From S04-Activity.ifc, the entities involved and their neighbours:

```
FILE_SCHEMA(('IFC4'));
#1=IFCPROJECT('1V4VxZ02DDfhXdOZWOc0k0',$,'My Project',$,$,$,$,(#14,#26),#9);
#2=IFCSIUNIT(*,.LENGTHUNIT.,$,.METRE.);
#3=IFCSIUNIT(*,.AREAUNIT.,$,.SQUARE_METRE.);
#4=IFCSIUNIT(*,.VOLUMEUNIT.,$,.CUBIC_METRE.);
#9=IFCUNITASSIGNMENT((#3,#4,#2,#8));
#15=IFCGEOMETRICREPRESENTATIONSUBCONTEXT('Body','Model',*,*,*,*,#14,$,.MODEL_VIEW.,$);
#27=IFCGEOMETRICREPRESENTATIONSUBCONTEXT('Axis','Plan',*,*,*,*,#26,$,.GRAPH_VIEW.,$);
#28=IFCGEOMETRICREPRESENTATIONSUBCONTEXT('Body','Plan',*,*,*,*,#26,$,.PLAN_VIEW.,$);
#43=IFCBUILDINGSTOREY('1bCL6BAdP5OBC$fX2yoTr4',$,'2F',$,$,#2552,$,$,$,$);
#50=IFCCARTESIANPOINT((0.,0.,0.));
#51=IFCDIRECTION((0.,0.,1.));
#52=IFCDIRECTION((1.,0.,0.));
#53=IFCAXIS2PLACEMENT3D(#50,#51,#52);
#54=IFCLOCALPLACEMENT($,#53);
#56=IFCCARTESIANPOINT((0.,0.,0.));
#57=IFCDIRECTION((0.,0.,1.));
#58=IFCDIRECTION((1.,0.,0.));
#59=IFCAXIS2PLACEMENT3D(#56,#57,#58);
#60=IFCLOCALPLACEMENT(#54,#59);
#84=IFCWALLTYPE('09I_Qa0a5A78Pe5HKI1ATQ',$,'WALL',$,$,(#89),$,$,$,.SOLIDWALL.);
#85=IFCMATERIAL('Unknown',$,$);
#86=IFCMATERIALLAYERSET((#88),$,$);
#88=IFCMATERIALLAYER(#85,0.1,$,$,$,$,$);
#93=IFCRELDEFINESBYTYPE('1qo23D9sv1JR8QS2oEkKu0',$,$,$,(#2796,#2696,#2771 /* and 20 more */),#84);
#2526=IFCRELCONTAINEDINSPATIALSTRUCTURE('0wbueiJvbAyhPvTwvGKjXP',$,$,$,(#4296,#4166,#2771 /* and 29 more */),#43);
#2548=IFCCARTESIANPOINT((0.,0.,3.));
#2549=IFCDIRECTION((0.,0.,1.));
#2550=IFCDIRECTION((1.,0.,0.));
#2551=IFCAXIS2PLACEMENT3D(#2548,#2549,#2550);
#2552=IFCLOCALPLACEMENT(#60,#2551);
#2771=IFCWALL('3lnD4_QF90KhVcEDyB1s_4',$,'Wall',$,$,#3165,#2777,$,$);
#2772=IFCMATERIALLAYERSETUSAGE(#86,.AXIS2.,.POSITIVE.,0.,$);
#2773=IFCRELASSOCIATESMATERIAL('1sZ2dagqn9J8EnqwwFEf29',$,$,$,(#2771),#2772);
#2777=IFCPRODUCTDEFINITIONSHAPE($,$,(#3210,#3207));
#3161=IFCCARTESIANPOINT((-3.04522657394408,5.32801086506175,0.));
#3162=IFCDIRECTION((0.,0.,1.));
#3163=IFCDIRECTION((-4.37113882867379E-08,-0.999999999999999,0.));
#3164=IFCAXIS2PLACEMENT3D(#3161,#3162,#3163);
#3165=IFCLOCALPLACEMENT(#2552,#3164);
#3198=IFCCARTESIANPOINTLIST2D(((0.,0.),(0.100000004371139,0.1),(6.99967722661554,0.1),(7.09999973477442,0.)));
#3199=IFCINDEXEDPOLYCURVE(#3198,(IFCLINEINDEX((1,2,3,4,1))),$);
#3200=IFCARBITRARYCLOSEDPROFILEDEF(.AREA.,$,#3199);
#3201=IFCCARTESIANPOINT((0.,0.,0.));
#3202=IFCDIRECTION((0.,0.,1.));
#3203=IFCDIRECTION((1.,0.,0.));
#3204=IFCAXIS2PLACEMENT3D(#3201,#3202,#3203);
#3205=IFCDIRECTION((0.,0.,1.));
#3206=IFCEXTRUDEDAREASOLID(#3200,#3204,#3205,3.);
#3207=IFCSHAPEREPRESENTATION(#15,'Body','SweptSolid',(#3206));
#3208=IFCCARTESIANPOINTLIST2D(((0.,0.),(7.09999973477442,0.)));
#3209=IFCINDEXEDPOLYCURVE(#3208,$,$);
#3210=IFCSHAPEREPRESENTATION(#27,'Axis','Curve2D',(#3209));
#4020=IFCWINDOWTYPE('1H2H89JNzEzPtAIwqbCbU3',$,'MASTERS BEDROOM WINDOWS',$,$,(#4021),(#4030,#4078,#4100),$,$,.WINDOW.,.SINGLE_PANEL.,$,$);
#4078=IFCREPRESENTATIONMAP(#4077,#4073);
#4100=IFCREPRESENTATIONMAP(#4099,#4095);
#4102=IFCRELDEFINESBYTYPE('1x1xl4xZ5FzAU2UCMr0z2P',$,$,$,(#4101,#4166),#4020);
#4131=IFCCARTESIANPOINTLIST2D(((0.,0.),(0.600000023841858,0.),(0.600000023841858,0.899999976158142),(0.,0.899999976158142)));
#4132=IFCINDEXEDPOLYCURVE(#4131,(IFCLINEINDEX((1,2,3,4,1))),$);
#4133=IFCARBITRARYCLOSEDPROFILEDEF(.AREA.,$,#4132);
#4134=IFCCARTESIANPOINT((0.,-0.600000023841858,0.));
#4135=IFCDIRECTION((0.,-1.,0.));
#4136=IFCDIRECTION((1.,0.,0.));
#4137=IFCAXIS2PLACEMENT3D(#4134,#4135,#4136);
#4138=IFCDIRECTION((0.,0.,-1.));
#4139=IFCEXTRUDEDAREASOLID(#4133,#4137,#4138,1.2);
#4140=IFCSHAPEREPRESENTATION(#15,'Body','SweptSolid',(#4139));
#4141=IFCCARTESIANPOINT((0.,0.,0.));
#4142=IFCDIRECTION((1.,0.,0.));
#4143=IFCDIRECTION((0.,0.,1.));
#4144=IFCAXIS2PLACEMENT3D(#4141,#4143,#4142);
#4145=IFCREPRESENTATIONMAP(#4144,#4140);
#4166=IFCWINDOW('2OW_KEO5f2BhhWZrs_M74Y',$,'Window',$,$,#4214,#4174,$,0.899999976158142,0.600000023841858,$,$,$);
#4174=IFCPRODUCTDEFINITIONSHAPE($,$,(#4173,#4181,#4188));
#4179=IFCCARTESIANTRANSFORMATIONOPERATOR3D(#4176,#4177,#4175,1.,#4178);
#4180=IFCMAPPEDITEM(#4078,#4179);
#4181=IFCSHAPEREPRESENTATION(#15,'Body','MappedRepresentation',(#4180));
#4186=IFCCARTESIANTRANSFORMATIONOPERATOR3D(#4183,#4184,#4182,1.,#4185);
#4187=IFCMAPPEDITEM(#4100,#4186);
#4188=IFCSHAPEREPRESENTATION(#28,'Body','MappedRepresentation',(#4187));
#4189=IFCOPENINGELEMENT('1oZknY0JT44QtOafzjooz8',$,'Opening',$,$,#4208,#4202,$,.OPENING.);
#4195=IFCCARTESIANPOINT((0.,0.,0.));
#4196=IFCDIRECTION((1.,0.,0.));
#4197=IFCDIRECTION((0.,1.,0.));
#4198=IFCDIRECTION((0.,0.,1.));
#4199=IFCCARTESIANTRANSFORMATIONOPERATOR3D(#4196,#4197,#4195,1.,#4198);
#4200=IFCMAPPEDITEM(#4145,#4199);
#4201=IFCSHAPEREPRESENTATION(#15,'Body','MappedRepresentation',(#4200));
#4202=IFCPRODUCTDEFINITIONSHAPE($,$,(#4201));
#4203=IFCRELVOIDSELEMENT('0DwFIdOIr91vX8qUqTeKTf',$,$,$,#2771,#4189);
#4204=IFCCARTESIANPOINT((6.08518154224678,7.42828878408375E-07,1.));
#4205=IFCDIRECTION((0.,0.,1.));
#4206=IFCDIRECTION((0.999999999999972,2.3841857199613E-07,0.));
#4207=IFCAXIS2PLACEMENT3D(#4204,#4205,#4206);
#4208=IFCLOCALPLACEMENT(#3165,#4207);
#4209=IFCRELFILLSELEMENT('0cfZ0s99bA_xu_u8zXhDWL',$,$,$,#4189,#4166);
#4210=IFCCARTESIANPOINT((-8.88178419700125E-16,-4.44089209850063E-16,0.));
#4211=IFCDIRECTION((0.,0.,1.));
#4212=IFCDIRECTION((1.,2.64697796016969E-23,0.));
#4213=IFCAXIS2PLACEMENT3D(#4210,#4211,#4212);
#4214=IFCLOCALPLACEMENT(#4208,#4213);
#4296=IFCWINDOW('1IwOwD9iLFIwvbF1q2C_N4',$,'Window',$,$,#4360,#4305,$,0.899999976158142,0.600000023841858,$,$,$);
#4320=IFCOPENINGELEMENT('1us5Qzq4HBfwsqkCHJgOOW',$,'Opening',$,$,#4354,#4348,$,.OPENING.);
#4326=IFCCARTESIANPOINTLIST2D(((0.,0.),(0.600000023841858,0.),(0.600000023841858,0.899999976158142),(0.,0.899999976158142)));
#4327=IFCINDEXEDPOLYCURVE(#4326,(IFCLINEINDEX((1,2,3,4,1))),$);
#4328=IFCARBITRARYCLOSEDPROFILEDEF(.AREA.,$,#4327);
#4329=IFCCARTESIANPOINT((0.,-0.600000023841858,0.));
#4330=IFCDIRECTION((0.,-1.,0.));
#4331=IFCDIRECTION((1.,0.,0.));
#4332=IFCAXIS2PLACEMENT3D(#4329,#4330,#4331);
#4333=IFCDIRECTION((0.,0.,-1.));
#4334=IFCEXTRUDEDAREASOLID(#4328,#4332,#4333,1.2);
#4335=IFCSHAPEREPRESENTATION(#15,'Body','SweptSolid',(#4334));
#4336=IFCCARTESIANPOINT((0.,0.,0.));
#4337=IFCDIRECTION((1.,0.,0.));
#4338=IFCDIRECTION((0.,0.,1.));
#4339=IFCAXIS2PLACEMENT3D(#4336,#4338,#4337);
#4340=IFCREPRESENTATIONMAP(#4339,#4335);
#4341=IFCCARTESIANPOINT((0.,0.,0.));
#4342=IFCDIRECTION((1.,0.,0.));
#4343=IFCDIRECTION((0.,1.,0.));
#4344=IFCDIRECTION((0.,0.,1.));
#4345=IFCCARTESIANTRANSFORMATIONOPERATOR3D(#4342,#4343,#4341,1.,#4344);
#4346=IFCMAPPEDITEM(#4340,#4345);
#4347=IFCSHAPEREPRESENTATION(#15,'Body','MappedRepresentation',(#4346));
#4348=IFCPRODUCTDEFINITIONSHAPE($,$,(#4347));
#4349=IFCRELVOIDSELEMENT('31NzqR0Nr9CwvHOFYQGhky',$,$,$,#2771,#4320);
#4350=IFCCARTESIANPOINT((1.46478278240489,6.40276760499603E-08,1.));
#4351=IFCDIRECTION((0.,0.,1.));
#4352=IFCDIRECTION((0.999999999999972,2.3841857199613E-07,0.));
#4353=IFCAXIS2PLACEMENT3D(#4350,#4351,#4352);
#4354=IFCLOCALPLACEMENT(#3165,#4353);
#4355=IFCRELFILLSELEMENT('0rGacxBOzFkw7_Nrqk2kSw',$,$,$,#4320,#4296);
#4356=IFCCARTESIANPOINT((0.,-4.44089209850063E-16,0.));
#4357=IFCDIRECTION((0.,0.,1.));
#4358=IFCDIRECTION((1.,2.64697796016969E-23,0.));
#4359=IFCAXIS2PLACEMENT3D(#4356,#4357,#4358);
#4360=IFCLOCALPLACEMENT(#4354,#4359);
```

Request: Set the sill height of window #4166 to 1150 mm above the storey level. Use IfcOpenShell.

```python
import numpy as np
import ifcopenshell
import ifcopenshell.api.geometry
import ifcopenshell.geom
import ifcopenshell.util.element
import ifcopenshell.util.placement
import ifcopenshell.util.shape
import ifcopenshell.util.unit

model = ifcopenshell.open("S04-Activity.ifc")
unit_scale = ifcopenshell.util.unit.calculate_unit_scale(model)

window = model.by_guid("2OW_KEO5f2BhhWZrs_M74Y")
opening = window.FillsVoids[0].RelatingOpeningElement
storey = ifcopenshell.util.element.get_container(window, ifc_class="IfcBuildingStorey")
level = ifcopenshell.util.placement.get_local_placement(storey.ObjectPlacement)[2, 3]

# The opening's origin need not be at the sill, so measure its lowest point.
shape = ifcopenshell.geom.create_shape(ifcopenshell.geom.settings(), opening)
bottom = ifcopenshell.util.shape.get_shape_bottom_elevation(shape, shape.geometry) / unit_scale
dz = level + 1.15 / unit_scale - bottom

shift = np.array([0.0, 0.0, dz])
# The window is placed relative to its opening, so it follows when the opening moves.
matrix = ifcopenshell.util.placement.get_local_placement(opening.ObjectPlacement)
matrix[:3, 3] += shift
ifcopenshell.api.geometry.edit_object_placement(
    model, product=opening, matrix=matrix, is_si=False, should_transform_children=True
)

print(f"moved by {dz * unit_scale:+.3f} m")

model.write("S04-Activity_v2.ifc")
```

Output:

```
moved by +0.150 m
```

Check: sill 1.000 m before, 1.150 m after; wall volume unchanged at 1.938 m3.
